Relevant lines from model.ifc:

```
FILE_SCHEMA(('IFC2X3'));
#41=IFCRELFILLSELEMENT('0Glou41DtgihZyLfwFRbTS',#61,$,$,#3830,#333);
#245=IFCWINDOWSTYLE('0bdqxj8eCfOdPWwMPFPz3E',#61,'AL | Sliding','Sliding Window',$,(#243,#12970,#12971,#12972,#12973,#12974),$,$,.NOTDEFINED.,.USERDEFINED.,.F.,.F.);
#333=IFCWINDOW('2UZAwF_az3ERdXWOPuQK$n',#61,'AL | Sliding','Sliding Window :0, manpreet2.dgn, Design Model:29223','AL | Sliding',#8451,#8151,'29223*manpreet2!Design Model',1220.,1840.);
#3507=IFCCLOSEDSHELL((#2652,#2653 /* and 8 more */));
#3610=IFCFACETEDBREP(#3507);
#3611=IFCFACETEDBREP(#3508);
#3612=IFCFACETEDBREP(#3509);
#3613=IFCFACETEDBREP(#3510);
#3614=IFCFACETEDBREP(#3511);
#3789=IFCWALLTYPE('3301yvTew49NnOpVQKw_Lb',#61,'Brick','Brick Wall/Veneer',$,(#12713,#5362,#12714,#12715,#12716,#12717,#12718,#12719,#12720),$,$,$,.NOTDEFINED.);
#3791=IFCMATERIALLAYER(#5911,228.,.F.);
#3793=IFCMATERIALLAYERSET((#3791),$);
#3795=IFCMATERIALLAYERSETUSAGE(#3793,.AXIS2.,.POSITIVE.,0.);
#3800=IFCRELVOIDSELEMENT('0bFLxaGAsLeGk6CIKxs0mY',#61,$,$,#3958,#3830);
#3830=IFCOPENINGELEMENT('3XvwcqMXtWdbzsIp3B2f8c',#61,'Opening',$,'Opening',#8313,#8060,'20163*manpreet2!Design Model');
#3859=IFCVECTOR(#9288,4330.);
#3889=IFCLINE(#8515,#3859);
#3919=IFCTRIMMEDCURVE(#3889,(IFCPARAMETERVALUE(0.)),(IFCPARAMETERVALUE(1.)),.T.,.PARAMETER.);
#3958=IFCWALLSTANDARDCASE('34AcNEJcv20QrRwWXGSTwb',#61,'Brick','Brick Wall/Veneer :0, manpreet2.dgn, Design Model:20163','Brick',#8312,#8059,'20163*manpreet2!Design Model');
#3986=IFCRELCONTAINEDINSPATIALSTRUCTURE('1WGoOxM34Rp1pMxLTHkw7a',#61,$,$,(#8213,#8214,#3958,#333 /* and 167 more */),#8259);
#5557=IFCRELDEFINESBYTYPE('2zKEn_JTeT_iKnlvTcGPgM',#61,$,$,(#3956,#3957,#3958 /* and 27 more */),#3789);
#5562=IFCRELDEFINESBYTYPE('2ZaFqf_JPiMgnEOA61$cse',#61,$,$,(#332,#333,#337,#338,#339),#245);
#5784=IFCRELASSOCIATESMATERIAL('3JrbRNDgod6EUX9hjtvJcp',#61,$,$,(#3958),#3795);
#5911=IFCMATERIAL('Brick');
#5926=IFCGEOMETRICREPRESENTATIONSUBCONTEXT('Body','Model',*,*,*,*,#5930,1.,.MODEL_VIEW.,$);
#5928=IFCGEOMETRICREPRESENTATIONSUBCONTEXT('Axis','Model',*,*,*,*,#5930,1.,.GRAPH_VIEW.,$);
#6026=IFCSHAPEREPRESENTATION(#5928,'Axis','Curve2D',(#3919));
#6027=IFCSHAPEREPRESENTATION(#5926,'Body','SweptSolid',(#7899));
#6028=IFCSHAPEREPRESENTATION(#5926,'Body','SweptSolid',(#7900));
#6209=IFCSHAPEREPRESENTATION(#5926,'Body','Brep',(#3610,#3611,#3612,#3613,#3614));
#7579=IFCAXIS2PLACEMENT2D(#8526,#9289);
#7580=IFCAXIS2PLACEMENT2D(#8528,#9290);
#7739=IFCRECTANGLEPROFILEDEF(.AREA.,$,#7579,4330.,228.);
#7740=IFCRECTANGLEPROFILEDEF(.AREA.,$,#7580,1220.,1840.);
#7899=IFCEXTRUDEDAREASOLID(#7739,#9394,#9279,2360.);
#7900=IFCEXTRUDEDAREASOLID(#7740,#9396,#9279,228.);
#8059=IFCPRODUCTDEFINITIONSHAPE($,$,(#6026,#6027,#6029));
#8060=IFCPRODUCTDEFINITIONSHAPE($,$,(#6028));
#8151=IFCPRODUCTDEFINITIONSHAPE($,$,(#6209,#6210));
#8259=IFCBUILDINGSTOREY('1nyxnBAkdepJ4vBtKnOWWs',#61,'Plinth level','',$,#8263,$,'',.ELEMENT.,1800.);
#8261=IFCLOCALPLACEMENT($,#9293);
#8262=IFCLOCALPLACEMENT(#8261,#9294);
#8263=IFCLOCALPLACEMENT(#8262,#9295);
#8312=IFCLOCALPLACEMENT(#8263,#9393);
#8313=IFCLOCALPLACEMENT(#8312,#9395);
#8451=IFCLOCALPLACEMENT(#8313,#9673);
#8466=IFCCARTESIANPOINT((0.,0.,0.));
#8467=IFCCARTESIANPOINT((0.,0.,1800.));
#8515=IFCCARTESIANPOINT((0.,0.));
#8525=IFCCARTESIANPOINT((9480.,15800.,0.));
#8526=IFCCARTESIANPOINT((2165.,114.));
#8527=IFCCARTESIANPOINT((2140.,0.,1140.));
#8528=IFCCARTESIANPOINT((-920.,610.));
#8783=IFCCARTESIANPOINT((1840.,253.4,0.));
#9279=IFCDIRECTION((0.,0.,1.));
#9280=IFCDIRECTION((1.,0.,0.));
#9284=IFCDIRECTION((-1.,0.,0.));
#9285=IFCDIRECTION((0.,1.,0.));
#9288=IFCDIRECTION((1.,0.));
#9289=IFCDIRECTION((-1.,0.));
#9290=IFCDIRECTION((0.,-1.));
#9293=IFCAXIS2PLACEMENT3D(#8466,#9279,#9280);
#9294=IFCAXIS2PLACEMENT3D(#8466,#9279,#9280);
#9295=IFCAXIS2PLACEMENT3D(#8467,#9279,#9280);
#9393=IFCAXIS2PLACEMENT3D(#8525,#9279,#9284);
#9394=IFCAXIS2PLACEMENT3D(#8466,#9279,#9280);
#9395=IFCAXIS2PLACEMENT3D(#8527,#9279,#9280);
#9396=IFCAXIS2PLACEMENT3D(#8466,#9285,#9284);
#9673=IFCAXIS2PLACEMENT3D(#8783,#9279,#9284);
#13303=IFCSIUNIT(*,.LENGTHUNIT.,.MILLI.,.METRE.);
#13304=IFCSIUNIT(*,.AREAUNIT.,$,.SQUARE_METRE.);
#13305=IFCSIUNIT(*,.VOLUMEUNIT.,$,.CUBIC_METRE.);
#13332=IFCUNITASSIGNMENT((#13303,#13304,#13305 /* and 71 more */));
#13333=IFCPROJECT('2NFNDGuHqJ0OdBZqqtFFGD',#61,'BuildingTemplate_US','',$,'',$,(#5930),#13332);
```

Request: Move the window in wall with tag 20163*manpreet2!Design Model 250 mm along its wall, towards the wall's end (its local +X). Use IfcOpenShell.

```python
import ifcopenshell
import ifcopenshell.api.geometry
import ifcopenshell.util.placement

model = ifcopenshell.open("model.ifc")

window = model.by_id(333)
opening = window.FillsVoids[0].RelatingOpeningElement
wall = opening.VoidsElements[0].RelatingBuildingElement

wall_matrix = ifcopenshell.util.placement.get_local_placement(wall.ObjectPlacement)
shift = wall_matrix[:3, 0] * 250.0
before = ifcopenshell.util.placement.get_local_placement(window.ObjectPlacement)[:3, 3].copy()

# The window is placed relative to its opening, so it follows when the opening moves.
matrix = ifcopenshell.util.placement.get_local_placement(opening.ObjectPlacement)
matrix[:3, 3] += shift
ifcopenshell.api.geometry.edit_object_placement(
    model, product=opening, matrix=matrix, is_si=False, should_transform_children=True
)

after = ifcopenshell.util.placement.get_local_placement(window.ObjectPlacement)[:3, 3]
print("window moved by", (after - before).round(3) + 0.0)

model.write("model_updated.ifc")
```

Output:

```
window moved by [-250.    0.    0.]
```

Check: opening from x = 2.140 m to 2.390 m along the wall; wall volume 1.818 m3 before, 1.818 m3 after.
